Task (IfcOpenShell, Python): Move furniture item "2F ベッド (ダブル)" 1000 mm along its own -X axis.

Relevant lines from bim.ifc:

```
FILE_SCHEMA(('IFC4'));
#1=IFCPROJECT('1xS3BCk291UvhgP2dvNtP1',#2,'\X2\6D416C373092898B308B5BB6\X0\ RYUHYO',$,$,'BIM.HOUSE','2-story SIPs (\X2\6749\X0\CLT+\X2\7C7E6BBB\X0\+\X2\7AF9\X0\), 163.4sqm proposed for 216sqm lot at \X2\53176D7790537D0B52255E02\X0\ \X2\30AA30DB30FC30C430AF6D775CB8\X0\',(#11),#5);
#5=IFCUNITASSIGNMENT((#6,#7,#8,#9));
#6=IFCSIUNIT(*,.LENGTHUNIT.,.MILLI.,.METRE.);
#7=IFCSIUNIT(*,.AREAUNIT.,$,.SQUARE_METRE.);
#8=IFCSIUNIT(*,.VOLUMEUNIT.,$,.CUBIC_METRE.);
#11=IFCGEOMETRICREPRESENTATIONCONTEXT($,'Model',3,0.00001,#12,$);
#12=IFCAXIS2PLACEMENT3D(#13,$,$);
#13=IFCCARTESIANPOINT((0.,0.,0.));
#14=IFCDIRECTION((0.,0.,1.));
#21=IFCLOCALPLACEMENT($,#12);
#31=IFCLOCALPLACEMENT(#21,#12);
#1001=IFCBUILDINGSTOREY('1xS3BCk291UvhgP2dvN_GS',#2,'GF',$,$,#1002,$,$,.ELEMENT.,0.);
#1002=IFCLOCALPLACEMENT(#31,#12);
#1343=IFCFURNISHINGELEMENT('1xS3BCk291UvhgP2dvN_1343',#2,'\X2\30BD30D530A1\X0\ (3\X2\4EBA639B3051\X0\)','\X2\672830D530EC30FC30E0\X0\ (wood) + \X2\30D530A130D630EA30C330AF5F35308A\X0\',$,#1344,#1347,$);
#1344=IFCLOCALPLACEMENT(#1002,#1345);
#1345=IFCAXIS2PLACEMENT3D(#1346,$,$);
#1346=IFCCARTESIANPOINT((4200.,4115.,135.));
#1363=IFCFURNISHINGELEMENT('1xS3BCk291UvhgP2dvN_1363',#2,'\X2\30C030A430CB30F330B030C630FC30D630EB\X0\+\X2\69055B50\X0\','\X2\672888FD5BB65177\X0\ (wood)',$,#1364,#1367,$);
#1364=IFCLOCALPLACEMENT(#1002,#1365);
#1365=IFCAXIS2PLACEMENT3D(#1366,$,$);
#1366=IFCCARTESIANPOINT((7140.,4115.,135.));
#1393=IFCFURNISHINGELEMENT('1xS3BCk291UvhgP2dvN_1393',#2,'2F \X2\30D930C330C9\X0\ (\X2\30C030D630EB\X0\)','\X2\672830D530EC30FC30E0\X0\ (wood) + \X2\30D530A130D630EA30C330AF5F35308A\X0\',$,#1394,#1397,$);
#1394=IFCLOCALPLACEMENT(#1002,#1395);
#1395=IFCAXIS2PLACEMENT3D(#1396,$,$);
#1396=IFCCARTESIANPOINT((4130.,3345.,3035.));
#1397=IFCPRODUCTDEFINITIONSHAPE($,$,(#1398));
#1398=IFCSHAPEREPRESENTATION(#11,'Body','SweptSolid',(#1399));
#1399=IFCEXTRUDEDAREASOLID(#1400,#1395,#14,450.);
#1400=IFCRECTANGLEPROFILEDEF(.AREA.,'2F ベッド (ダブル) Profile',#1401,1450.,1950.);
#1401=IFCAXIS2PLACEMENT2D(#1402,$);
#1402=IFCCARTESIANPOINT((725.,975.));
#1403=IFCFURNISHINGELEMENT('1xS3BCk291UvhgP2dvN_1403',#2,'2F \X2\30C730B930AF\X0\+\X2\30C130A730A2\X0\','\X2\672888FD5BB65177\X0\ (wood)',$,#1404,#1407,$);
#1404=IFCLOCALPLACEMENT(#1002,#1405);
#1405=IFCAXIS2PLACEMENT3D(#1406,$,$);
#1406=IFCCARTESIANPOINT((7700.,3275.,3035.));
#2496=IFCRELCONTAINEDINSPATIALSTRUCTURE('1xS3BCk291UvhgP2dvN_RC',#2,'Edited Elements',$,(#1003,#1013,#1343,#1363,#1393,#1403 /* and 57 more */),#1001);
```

```python
import ifcopenshell
import ifcopenshell.api.geometry
import ifcopenshell.util.placement
import ifcopenshell.util.unit

model = ifcopenshell.open("bim.ifc")
unit_scale = ifcopenshell.util.unit.calculate_unit_scale(model)

item = model.by_id(1393)
matrix = ifcopenshell.util.placement.get_local_placement(item.ObjectPlacement)
matrix[:3, 3] -= matrix[:3, 0] * 1 / unit_scale
ifcopenshell.api.geometry.edit_object_placement(model, product=item, matrix=matrix, is_si=False)

print(ifcopenshell.util.placement.get_local_placement(item.ObjectPlacement).round(3) + 0.0)

model.write("bim_v2.ifc")
```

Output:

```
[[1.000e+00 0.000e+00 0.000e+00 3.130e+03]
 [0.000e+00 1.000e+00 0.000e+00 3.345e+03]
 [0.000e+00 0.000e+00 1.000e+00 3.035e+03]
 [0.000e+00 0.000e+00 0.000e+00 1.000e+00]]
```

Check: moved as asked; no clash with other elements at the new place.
